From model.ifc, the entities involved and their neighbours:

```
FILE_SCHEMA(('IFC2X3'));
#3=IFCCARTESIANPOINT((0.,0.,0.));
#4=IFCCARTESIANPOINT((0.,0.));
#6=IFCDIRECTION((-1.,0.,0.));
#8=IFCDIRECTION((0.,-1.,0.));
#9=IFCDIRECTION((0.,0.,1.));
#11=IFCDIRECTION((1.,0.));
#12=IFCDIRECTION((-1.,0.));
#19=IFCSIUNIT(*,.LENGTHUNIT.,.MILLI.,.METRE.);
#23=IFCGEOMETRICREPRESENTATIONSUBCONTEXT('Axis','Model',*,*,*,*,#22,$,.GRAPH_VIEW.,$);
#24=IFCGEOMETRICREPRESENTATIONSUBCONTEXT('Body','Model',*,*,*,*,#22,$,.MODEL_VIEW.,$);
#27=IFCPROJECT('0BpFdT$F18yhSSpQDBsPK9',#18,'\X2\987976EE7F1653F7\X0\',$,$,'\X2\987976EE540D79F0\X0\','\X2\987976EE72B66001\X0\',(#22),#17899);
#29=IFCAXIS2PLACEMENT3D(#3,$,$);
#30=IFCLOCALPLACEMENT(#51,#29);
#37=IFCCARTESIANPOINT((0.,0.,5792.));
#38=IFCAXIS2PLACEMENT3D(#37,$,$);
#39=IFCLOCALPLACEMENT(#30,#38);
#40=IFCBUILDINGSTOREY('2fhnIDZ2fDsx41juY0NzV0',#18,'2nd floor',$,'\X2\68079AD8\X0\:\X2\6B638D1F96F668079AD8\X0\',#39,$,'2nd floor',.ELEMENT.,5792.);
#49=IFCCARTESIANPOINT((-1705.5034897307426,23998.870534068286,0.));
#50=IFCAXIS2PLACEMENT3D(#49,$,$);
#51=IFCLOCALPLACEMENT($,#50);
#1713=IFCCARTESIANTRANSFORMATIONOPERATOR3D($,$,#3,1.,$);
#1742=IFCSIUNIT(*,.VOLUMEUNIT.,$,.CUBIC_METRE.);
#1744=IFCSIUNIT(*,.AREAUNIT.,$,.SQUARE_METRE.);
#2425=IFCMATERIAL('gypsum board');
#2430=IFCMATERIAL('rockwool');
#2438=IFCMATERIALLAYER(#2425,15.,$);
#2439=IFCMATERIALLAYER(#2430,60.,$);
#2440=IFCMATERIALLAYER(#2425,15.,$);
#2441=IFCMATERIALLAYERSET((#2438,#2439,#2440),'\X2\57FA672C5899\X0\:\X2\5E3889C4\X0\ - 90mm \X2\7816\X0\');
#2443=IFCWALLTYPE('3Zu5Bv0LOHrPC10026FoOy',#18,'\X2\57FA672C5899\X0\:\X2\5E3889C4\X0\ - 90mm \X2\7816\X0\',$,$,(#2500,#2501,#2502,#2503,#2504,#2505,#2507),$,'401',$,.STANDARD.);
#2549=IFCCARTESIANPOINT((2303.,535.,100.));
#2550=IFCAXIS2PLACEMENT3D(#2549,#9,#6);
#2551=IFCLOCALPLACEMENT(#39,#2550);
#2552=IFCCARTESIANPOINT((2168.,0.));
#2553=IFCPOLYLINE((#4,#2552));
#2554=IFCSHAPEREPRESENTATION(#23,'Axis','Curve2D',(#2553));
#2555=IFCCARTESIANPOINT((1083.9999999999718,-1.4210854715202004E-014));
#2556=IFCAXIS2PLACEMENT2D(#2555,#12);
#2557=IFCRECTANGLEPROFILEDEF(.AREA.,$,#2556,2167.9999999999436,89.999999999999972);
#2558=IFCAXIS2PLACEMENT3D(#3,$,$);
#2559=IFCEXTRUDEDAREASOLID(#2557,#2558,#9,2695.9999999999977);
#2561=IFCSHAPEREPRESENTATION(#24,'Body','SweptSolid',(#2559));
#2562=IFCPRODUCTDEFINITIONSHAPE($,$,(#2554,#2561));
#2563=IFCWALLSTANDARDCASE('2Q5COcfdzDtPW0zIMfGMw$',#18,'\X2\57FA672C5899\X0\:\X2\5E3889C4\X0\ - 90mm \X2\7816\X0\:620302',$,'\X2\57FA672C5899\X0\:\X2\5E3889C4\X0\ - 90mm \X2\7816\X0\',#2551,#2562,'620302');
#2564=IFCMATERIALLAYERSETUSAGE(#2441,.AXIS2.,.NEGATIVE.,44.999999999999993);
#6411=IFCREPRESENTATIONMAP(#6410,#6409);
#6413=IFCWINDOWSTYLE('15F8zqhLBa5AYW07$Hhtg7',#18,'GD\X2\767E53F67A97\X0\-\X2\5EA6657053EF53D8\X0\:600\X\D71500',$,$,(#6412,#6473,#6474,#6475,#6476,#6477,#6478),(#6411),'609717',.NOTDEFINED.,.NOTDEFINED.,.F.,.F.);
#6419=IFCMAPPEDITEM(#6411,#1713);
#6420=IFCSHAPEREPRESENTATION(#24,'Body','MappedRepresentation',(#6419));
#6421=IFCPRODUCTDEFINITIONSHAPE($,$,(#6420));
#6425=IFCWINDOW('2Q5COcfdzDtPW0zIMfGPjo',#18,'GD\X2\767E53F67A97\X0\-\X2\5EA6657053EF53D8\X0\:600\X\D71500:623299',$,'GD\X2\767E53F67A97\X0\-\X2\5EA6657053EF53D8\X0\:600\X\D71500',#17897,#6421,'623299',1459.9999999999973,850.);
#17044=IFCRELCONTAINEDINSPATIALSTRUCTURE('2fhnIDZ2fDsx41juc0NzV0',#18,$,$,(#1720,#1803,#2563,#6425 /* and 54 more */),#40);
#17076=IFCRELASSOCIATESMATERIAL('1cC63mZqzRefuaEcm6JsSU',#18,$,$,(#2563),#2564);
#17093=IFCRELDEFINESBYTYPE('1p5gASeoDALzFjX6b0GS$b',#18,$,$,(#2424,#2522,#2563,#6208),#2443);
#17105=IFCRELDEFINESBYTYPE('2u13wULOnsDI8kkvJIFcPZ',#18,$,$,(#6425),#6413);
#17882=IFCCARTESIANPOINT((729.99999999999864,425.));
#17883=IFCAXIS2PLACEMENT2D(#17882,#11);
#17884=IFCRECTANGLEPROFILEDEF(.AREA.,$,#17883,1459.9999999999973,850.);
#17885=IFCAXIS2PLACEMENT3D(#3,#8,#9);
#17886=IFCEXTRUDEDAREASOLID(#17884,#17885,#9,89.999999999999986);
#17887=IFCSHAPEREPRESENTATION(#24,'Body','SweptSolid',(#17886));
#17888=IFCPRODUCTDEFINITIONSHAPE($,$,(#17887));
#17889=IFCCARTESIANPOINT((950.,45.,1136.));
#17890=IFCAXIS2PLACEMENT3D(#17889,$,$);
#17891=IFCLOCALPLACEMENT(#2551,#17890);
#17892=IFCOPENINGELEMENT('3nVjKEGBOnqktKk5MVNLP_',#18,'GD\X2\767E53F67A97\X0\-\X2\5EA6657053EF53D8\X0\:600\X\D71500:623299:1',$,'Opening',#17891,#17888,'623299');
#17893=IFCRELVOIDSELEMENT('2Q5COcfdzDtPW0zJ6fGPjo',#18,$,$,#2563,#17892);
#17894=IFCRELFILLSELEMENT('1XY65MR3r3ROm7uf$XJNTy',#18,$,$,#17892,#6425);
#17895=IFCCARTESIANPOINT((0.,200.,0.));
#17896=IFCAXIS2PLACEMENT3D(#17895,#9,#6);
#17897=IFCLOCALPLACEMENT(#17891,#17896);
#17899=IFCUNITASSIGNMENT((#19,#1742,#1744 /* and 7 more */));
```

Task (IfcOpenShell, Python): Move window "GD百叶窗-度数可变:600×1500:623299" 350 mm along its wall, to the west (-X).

```python
import ifcopenshell
import ifcopenshell.api.geometry
import ifcopenshell.util.placement
import ifcopenshell.util.unit

model = ifcopenshell.open("model.ifc")
unit_scale = ifcopenshell.util.unit.calculate_unit_scale(model)

window = model.by_guid("2Q5COcfdzDtPW0zIMfGPjo")
opening = window.FillsVoids[0].RelatingOpeningElement
wall = opening.VoidsElements[0].RelatingBuildingElement

wall_matrix = ifcopenshell.util.placement.get_local_placement(wall.ObjectPlacement)
shift = wall_matrix[:3, 0] * 0.35 / unit_scale
before = ifcopenshell.util.placement.get_local_placement(window.ObjectPlacement)[:3, 3].copy()

# The window is placed relative to its opening, so it follows when the opening moves.
matrix = ifcopenshell.util.placement.get_local_placement(opening.ObjectPlacement)
matrix[:3, 3] += shift
ifcopenshell.api.geometry.edit_object_placement(
    model, product=opening, matrix=matrix, is_si=False, should_transform_children=True
)

after = ifcopenshell.util.placement.get_local_placement(window.ObjectPlacement)[:3, 3]
print("window moved by", (after - before).round(3) + 0.0)

model.write("model_edited.ifc")
```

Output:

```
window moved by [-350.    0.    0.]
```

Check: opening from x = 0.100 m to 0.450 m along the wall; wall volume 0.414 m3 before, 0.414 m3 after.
